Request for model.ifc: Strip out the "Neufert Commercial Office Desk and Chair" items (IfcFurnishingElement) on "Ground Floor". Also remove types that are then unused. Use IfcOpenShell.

First a look at what the model holds.

```python
import ifcopenshell
import ifcopenshell.util.element

model = ifcopenshell.open("model.ifc")
print(model.schema)
storey = next(s for s in model.by_type("IfcBuildingStorey") if s.Name == "Ground Floor")
furniture = [e for e in ifcopenshell.util.element.get_decomposition(storey) if e.is_a("IfcFurnishingElement")]
seen = {}
for e in furniture:
    element_type = ifcopenshell.util.element.get_type(e)
    name = element_type.Name if element_type not in (None, e) else None
    seen[name] = seen.get(name, 0) + 1
for name, count in sorted(seen.items(), key=str):
    print(count, "x", name)
```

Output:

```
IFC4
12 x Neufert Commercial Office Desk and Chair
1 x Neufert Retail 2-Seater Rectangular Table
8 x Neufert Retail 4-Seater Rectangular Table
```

```python
import ifcopenshell
import ifcopenshell.api.root
import ifcopenshell.util.element

model = ifcopenshell.open("model.ifc")

storey = next(s for s in model.by_type("IfcBuildingStorey") if s.Name == "Ground Floor")
furniture = [e for e in ifcopenshell.util.element.get_decomposition(storey) if e.is_a("IfcFurnishingElement")]
targets = [e for e in furniture if (t := ifcopenshell.util.element.get_type(e)) not in (None, e) and t.Name == "Neufert Commercial Office Desk and Chair"]
types = {ifcopenshell.util.element.get_type(e) for e in targets} - {None, *targets}

for e in targets:
    ifcopenshell.api.root.remove_product(model, product=e)
print(len(targets), "removed")

unused = [t for t in types if not ifcopenshell.util.element.get_types(t)]
for t in unused:
    ifcopenshell.api.root.remove_product(model, product=t)
print(len(unused), "unused types removed")

model.write("model_edited.ifc")
```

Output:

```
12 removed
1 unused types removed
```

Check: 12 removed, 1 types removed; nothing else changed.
